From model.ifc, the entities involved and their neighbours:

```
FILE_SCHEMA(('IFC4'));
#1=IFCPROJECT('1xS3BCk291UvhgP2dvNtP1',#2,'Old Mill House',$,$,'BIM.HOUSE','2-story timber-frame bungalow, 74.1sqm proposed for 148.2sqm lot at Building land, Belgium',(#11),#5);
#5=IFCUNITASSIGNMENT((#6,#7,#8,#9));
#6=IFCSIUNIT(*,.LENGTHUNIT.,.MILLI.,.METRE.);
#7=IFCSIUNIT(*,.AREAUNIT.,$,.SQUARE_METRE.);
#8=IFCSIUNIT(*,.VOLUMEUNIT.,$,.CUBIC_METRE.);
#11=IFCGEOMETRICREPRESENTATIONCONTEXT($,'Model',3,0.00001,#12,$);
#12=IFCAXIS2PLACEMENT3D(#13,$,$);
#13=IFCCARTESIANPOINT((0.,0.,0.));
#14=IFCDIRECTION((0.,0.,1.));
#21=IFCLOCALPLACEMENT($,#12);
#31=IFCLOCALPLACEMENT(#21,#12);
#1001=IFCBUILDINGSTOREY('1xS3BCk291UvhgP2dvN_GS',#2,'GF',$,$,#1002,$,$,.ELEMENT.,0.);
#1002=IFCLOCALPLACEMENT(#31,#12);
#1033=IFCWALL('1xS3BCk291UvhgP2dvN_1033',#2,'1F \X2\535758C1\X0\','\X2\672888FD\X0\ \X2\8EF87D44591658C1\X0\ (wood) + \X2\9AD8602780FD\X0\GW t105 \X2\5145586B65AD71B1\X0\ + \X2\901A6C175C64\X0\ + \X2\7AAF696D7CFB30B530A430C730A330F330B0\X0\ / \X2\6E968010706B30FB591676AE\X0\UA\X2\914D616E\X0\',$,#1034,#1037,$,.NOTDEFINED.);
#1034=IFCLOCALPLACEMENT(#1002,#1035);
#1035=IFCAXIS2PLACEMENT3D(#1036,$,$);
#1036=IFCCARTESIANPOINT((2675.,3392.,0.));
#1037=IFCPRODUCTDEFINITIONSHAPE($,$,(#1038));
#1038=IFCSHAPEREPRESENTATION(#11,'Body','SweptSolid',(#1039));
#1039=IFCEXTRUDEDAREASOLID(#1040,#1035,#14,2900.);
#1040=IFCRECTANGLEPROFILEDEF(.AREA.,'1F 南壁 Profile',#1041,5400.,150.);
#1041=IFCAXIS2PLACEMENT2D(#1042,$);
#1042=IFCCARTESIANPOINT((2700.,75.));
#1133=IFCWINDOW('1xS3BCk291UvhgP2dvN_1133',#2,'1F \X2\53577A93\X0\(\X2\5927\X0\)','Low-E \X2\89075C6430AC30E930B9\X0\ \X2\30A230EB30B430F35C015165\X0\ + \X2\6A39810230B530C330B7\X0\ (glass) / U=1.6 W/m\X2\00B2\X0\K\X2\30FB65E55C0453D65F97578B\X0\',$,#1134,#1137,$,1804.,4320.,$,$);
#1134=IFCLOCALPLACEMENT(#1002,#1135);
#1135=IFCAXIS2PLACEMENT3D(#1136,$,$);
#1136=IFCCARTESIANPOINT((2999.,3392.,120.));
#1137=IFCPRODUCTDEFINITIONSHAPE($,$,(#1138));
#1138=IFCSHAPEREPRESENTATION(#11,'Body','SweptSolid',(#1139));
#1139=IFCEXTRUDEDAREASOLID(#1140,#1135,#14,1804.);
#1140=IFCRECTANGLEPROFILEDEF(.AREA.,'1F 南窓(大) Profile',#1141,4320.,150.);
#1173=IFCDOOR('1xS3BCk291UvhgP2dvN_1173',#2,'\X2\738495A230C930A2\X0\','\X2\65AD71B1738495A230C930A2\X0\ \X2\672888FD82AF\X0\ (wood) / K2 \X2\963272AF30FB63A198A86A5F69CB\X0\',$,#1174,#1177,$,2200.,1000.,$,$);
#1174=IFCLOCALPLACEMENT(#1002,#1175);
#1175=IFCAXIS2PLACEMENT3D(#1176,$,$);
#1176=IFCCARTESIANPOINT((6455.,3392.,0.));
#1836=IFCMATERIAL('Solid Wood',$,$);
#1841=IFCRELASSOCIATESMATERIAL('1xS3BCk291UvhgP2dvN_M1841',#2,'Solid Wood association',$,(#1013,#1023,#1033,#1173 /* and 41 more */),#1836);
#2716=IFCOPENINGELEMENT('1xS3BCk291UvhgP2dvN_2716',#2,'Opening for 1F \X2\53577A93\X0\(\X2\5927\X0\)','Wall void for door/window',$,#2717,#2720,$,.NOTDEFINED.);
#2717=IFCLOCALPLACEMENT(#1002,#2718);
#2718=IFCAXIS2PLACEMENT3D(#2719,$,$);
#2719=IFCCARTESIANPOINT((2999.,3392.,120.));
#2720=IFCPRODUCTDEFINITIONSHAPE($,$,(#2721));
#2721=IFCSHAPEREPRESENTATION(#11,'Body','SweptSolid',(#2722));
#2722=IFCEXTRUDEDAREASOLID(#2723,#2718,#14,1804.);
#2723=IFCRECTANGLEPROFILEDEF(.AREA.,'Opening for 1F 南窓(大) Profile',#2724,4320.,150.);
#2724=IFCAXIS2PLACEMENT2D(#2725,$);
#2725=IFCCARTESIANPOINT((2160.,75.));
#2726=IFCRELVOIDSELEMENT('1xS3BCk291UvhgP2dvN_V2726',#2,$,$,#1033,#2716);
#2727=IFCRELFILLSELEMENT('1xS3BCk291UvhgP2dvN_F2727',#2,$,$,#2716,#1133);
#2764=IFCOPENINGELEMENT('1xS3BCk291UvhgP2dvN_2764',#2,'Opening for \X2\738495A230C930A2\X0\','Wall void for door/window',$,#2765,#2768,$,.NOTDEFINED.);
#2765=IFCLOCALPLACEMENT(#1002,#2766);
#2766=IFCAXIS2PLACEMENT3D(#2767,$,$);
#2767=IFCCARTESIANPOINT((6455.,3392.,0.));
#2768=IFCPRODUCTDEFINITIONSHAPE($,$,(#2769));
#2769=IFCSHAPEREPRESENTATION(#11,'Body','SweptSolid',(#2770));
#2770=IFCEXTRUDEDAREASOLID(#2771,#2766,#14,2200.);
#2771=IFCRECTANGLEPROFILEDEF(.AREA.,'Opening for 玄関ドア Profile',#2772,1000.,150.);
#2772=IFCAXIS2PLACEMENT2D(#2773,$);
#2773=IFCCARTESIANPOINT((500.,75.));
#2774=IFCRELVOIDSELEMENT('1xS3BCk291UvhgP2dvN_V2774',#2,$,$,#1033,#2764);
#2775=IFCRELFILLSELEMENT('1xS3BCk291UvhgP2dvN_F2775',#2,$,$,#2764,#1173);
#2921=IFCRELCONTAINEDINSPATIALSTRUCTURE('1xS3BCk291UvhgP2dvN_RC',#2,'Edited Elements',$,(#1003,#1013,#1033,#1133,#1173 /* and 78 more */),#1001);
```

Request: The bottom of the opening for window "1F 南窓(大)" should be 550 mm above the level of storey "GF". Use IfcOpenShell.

```python
import numpy as np
import ifcopenshell
import ifcopenshell.api.geometry
import ifcopenshell.geom
import ifcopenshell.util.element
import ifcopenshell.util.placement
import ifcopenshell.util.shape
import ifcopenshell.util.unit

model = ifcopenshell.open("model.ifc")
unit_scale = ifcopenshell.util.unit.calculate_unit_scale(model)

window = model.by_id(1133)
opening = window.FillsVoids[0].RelatingOpeningElement
storey = ifcopenshell.util.element.get_container(window, ifc_class="IfcBuildingStorey")
level = ifcopenshell.util.placement.get_local_placement(storey.ObjectPlacement)[2, 3]

# The opening's origin need not be at the sill, so measure its lowest point.
shape = ifcopenshell.geom.create_shape(ifcopenshell.geom.settings(), opening)
bottom = ifcopenshell.util.shape.get_shape_bottom_elevation(shape, shape.geometry) / unit_scale
dz = level + 550.0 - bottom

shift = np.array([0.0, 0.0, dz])
# The window is not placed relative to its opening, so move both.
for product in (opening, window):
    matrix = ifcopenshell.util.placement.get_local_placement(product.ObjectPlacement)
    matrix[:3, 3] += shift
    ifcopenshell.api.geometry.edit_object_placement(model, product=product, matrix=matrix, is_si=False)

print(f"moved by {dz * unit_scale:+.3f} m")

model.write("model_rev.ifc")
```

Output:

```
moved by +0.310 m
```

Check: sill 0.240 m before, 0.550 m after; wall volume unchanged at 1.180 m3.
